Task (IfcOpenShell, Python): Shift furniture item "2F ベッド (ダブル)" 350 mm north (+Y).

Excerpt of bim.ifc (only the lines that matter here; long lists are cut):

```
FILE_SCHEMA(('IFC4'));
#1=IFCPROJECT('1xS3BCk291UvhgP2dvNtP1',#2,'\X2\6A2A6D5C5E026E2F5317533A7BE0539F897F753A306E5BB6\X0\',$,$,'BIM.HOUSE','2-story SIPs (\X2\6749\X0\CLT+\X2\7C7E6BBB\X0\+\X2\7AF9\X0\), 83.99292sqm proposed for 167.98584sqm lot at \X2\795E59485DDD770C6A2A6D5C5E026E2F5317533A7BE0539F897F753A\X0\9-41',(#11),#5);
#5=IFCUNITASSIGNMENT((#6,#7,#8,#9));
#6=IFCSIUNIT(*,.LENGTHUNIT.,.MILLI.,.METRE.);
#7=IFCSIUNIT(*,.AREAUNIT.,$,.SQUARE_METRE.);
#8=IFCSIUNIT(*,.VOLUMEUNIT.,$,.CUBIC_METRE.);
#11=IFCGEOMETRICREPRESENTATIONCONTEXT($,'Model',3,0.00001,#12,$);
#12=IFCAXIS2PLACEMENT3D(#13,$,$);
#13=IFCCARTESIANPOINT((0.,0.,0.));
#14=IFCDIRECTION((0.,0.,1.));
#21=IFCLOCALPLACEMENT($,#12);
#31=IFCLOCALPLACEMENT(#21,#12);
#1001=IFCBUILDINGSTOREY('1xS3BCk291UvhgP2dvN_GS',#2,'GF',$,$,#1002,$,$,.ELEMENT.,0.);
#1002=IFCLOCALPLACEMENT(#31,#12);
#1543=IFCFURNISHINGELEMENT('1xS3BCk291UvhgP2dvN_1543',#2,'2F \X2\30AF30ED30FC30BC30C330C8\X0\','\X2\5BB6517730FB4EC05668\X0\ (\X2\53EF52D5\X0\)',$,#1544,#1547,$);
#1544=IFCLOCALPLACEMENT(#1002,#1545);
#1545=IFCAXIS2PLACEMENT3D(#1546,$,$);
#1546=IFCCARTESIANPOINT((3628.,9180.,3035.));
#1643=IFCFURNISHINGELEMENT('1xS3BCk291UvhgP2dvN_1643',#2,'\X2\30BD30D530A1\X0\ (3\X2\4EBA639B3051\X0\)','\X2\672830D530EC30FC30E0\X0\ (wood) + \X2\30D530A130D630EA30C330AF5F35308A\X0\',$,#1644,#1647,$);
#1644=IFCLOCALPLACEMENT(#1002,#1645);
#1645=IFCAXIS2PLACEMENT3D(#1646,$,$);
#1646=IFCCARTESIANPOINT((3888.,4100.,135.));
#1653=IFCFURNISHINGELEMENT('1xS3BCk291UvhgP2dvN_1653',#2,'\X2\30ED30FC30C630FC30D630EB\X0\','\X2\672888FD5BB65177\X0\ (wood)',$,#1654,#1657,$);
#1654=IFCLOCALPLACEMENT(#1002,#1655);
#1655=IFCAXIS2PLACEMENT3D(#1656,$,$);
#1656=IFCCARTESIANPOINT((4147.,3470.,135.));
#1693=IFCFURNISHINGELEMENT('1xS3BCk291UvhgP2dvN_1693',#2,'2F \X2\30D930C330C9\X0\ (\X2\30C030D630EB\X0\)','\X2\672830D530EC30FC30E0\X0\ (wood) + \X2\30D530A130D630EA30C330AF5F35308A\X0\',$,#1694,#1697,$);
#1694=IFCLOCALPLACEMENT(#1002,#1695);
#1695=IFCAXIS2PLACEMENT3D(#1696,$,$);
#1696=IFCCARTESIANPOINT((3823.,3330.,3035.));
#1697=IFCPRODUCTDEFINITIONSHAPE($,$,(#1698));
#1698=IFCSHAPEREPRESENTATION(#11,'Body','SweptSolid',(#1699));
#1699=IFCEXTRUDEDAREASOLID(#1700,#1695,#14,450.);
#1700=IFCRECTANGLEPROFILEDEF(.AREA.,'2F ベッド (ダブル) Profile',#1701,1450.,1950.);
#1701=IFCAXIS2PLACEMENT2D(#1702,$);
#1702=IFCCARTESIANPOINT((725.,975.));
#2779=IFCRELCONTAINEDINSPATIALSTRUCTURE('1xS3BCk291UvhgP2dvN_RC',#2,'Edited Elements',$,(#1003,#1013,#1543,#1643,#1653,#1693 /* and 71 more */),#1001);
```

```python
import ifcopenshell
import ifcopenshell.api.geometry
import ifcopenshell.util.placement
import ifcopenshell.util.unit

model = ifcopenshell.open("bim.ifc")
unit_scale = ifcopenshell.util.unit.calculate_unit_scale(model)

item = model.by_guid("1xS3BCk291UvhgP2dvN_1693")
matrix = ifcopenshell.util.placement.get_local_placement(item.ObjectPlacement)
matrix[1, 3] += 0.35 / unit_scale
ifcopenshell.api.geometry.edit_object_placement(model, product=item, matrix=matrix, is_si=False)

print(ifcopenshell.util.placement.get_local_placement(item.ObjectPlacement).round(3) + 0.0)

model.write("bim_edited.ifc")
```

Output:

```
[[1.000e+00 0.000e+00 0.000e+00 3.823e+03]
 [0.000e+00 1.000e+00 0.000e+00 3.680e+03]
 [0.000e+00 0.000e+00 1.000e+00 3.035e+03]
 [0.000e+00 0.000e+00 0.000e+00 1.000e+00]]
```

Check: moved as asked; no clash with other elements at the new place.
